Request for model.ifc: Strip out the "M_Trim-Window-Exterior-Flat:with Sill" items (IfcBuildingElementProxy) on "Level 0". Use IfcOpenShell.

First a look at what the model holds.

```python
import ifcopenshell
import ifcopenshell.util.element

model = ifcopenshell.open("model.ifc")
print(model.schema)
storey = next(s for s in model.by_type("IfcBuildingStorey") if s.Name == "Level 0")
proxies = [e for e in ifcopenshell.util.element.get_decomposition(storey) if e.is_a("IfcBuildingElementProxy")]
seen = {}
for e in proxies:
    element_type = ifcopenshell.util.element.get_type(e)
    name = element_type.Name if element_type not in (None, e) else None
    seen[name] = seen.get(name, 0) + 1
for name, count in sorted(seen.items(), key=str):
    print(count, "x", name)
```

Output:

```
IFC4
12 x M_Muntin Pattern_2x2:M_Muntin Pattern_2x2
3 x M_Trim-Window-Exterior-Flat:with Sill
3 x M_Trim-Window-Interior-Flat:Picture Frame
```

```python
import ifcopenshell
import ifcopenshell.api.root
import ifcopenshell.util.element

model = ifcopenshell.open("model.ifc")

storey = next(s for s in model.by_type("IfcBuildingStorey") if s.Name == "Level 0")
proxies = [e for e in ifcopenshell.util.element.get_decomposition(storey) if e.is_a("IfcBuildingElementProxy")]
targets = [e for e in proxies if (t := ifcopenshell.util.element.get_type(e)) not in (None, e) and t.Name == "M_Trim-Window-Exterior-Flat:with Sill"]

for e in targets:
    ifcopenshell.api.root.remove_product(model, product=e)
print(len(targets), "removed")

model.write("model_rev.ifc")
```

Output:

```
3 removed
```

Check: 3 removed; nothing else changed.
